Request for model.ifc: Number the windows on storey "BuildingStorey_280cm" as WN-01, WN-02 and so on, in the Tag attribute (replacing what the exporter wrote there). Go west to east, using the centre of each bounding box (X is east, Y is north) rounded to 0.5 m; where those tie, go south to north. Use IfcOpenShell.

First a look at what the model holds.

```python
import ifcopenshell
import ifcopenshell.util.element
import ifcopenshell.util.placement

model = ifcopenshell.open("model.ifc")
print(model.schema)
storey = next(s for s in model.by_type("IfcBuildingStorey") if s.Name == "BuildingStorey_280cm")
windows = [e for e in ifcopenshell.util.element.get_decomposition(storey) if e.is_a("IfcWindow")]
for e in sorted(windows, key=lambda e: e.id()):
    origin = ifcopenshell.util.placement.get_local_placement(e.ObjectPlacement)[:3, 3]
    print(e.id(), e.Tag, e.Name, origin.round(2) + 0.0, sep=" | ")
```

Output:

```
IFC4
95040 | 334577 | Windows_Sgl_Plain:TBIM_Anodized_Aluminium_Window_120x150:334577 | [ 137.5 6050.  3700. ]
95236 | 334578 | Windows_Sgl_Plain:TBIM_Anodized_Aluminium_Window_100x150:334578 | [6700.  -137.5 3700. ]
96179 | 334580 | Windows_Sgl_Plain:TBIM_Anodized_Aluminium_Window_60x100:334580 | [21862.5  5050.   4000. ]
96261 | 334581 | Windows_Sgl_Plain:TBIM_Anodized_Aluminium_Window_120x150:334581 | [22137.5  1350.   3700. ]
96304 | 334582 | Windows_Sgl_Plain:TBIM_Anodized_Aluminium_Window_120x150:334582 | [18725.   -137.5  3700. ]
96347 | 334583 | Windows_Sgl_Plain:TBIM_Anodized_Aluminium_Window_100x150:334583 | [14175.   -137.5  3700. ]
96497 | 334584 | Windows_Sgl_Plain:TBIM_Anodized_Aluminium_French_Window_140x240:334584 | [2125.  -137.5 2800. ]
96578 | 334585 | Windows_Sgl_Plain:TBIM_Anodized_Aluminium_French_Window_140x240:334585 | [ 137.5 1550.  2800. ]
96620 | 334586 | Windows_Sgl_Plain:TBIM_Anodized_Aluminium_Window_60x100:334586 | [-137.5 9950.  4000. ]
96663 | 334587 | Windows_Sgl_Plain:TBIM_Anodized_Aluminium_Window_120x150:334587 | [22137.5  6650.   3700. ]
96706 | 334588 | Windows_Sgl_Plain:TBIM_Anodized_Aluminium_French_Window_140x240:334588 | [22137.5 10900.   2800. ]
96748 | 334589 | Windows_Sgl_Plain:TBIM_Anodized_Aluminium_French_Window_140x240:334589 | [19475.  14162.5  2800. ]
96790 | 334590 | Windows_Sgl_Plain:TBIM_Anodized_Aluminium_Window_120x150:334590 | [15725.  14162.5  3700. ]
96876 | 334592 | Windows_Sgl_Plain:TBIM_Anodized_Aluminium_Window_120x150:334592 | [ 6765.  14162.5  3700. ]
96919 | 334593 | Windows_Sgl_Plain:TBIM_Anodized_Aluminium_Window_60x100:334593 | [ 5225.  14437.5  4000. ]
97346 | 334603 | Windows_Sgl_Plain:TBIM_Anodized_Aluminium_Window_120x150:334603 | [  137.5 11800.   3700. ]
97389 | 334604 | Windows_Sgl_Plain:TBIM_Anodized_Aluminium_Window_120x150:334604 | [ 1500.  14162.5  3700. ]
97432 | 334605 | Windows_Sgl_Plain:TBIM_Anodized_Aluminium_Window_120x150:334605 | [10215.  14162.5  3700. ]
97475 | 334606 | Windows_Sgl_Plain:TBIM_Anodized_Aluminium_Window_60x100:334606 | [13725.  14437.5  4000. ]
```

```python
import ifcopenshell
import ifcopenshell.geom
import ifcopenshell.util.element
import ifcopenshell.util.shape

model = ifcopenshell.open("model.ifc")
settings = ifcopenshell.geom.settings()
settings.set("use-world-coords", True)


def centre(element):
    shape = ifcopenshell.geom.create_shape(settings, element)
    return ifcopenshell.util.shape.get_bbox_centroid(shape.geometry)


storey = next(s for s in model.by_type("IfcBuildingStorey") if s.Name == "BuildingStorey_280cm")
windows = [e for e in ifcopenshell.util.element.get_decomposition(storey) if e.is_a("IfcWindow")]

# Insertion points can sit at a corner or the storey origin, so sort by the geometry (in metres).
centres = {e: centre(e) for e in windows}
windows.sort(key=lambda e: (round(centres[e][0] / 0.5), centres[e][1]))

for i, e in enumerate(windows, start=1):
    number = f"WN-{i:02d}"
    e.Tag = number
    print(e.id(), number)

model.write("model_v2.ifc")
```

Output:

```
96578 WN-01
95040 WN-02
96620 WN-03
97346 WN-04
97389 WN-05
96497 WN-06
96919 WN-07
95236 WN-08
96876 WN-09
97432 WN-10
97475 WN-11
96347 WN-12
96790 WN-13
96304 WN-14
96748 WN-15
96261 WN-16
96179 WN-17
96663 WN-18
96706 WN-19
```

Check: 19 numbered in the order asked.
